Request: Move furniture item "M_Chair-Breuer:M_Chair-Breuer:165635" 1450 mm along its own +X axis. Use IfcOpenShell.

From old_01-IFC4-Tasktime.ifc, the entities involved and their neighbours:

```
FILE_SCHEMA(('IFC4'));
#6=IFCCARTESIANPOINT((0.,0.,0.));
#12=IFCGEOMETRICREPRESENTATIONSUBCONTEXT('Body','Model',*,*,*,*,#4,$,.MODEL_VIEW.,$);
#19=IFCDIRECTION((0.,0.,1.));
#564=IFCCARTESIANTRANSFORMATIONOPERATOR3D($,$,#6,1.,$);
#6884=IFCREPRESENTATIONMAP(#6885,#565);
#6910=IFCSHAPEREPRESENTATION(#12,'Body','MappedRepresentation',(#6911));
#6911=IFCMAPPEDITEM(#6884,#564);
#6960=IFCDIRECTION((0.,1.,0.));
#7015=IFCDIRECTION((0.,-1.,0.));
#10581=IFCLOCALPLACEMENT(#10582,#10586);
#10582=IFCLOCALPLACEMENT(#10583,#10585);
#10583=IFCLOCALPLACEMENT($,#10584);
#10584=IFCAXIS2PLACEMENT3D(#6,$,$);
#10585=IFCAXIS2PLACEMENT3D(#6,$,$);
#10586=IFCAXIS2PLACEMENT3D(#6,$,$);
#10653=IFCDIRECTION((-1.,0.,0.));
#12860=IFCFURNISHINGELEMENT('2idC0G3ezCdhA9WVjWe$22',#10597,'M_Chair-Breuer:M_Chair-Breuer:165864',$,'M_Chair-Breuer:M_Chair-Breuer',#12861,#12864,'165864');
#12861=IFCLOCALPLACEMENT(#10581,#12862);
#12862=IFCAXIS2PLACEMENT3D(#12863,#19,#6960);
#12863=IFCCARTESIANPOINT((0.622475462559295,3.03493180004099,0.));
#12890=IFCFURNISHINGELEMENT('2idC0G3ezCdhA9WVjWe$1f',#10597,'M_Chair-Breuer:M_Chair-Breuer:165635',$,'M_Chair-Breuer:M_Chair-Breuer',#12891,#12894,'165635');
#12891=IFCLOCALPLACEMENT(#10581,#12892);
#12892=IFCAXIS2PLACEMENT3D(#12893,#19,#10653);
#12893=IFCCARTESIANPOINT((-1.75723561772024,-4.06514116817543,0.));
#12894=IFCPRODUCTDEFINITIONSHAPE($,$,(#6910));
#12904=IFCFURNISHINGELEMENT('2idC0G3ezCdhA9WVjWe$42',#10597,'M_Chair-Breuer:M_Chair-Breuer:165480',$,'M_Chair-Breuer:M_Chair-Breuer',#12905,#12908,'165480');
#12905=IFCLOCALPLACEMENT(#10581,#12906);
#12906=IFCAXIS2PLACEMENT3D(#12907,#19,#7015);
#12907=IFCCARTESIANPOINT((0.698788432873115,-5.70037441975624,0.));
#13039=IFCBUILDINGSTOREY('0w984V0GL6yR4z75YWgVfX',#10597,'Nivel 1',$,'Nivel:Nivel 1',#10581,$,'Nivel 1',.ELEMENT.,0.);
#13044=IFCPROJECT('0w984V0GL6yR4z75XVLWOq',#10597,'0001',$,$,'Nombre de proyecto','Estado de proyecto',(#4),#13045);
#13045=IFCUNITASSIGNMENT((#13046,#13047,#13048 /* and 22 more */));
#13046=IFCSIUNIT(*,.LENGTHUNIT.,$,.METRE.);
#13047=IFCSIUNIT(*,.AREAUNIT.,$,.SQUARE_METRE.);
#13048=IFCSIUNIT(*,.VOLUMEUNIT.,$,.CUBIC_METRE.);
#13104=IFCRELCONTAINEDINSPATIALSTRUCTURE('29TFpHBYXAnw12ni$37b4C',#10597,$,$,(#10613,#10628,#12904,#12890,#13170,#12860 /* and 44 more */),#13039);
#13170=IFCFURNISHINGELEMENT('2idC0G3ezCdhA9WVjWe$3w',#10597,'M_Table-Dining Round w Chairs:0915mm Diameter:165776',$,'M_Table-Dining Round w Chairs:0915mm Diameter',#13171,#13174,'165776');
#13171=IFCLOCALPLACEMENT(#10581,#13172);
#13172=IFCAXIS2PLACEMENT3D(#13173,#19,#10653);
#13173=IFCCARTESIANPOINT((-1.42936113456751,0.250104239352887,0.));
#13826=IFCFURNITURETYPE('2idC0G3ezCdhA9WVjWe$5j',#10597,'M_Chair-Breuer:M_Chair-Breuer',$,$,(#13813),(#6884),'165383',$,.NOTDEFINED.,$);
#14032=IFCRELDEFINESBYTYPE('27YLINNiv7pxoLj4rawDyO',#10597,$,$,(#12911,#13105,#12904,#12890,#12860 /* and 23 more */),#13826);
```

```python
import ifcopenshell
import ifcopenshell.api.geometry
import ifcopenshell.util.placement
import ifcopenshell.util.unit

model = ifcopenshell.open("old_01-IFC4-Tasktime.ifc")
unit_scale = ifcopenshell.util.unit.calculate_unit_scale(model)

item = model.by_guid("2idC0G3ezCdhA9WVjWe$1f")
matrix = ifcopenshell.util.placement.get_local_placement(item.ObjectPlacement)
matrix[:3, 3] += matrix[:3, 0] * 1.45 / unit_scale
ifcopenshell.api.geometry.edit_object_placement(model, product=item, matrix=matrix, is_si=False)

print(ifcopenshell.util.placement.get_local_placement(item.ObjectPlacement).round(3) + 0.0)

model.write("old_01-IFC4-Tasktime_updated.ifc")
```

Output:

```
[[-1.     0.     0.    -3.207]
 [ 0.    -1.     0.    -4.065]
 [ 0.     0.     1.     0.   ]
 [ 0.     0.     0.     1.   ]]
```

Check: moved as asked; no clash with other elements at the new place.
